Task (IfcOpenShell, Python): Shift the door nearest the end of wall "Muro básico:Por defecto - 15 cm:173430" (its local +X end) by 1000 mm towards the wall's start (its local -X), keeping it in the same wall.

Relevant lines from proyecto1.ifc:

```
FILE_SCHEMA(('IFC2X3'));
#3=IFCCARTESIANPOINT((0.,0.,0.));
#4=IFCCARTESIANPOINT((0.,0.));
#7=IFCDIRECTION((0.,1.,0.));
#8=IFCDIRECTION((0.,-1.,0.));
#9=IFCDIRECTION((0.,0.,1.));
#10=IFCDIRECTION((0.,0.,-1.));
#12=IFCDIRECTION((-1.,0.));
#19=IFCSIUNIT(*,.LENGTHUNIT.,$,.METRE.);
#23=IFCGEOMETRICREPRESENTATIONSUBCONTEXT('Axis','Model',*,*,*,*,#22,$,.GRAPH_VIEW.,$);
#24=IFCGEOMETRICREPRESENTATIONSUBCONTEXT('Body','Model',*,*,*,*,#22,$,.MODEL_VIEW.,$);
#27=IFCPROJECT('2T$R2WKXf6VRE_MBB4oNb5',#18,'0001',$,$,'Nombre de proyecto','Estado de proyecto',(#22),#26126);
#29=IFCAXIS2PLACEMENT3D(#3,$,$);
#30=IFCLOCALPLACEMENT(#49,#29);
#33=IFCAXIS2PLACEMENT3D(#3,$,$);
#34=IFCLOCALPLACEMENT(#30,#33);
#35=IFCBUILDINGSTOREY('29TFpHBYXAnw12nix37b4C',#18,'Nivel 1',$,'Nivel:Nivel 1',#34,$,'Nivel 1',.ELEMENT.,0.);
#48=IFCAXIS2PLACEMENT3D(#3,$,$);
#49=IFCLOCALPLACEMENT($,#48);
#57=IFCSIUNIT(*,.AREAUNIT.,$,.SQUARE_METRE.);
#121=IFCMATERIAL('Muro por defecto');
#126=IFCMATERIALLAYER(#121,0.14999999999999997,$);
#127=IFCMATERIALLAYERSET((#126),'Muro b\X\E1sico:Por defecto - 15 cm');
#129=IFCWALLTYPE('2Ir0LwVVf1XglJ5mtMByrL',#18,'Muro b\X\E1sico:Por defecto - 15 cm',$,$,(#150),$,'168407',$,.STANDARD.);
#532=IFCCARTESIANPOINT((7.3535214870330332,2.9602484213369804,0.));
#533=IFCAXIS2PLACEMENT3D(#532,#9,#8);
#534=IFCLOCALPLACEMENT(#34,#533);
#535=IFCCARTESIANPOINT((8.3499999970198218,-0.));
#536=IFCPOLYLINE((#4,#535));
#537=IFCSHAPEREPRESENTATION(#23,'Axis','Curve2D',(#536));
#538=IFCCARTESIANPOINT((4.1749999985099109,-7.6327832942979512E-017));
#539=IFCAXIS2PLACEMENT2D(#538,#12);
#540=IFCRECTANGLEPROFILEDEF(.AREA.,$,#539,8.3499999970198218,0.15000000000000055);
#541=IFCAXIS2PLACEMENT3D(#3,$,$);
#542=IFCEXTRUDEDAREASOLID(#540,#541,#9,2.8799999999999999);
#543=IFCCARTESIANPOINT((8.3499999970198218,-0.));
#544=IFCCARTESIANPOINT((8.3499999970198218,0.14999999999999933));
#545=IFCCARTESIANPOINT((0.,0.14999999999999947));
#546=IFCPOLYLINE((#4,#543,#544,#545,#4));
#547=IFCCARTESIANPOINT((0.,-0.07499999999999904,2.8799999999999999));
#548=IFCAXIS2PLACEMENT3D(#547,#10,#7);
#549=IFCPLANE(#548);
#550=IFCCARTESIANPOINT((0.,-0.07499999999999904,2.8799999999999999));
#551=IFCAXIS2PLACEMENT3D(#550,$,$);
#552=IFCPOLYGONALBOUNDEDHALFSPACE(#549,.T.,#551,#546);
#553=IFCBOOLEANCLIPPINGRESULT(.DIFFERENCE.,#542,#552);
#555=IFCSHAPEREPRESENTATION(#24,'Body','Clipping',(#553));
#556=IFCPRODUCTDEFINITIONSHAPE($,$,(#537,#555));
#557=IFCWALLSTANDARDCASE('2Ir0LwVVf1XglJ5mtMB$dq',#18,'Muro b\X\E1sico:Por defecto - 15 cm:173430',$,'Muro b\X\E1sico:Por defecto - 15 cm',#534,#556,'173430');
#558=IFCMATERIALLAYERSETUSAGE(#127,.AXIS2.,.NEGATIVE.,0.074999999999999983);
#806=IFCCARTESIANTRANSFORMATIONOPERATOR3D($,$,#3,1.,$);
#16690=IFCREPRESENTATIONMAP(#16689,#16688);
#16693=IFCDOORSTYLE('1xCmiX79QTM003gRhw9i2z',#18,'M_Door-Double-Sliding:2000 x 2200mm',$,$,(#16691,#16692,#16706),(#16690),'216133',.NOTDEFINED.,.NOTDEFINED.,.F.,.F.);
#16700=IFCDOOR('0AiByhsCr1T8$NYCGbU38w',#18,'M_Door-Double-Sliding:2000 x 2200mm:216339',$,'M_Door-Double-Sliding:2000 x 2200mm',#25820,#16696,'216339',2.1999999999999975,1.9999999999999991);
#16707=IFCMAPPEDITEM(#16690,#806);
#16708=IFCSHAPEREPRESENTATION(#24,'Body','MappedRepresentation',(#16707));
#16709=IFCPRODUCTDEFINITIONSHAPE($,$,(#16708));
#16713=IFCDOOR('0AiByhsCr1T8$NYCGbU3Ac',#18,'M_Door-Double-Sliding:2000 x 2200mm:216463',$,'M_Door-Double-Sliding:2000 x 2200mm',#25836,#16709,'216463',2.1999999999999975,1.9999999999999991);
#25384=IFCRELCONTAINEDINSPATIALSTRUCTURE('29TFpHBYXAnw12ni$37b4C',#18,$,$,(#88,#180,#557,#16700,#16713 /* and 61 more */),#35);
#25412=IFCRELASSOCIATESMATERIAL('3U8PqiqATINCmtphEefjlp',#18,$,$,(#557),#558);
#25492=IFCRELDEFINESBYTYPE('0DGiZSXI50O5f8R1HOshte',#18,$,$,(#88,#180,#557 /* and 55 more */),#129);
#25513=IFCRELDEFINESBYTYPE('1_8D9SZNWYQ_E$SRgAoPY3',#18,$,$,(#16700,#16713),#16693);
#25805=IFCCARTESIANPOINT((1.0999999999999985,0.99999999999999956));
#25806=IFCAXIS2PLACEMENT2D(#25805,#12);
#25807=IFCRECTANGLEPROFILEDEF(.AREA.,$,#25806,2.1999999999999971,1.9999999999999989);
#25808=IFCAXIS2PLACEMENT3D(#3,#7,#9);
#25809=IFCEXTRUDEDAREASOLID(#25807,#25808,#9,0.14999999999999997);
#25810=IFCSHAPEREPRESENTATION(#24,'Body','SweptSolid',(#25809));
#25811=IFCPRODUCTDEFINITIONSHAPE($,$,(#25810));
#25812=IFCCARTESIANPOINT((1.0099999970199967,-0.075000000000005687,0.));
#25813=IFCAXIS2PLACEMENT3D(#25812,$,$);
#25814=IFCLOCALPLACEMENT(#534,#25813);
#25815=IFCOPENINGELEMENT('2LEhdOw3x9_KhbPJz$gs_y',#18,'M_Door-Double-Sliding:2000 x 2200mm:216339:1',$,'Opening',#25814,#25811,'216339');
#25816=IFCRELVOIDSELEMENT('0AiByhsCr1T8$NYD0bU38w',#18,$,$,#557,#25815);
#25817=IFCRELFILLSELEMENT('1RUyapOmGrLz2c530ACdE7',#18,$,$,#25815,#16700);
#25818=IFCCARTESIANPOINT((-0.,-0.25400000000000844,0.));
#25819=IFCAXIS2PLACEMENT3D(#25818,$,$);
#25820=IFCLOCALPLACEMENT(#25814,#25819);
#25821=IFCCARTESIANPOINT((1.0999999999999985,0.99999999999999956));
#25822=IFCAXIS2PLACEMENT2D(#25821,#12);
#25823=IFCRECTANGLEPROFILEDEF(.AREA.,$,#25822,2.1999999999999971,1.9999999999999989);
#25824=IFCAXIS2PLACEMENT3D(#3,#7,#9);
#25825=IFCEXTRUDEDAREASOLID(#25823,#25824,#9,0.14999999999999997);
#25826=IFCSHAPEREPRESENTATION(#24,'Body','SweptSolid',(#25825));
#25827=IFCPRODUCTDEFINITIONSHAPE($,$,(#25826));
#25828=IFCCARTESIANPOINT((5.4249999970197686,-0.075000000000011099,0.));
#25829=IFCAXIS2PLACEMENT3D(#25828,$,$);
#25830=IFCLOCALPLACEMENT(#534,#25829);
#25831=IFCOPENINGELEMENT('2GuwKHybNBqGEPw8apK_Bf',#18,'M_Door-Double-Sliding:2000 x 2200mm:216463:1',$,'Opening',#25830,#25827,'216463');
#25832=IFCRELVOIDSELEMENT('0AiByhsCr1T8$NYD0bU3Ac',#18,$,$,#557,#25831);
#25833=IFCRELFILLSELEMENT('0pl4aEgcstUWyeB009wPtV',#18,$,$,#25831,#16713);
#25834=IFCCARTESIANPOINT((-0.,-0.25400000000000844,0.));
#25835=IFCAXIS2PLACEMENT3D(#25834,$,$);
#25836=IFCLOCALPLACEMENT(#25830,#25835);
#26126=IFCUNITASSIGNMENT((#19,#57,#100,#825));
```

```python
import ifcopenshell
import ifcopenshell.api.geometry
import ifcopenshell.util.placement
import ifcopenshell.util.unit

model = ifcopenshell.open("proyecto1.ifc")
unit_scale = ifcopenshell.util.unit.calculate_unit_scale(model)

door = model.by_guid("0AiByhsCr1T8$NYCGbU3Ac")
opening = door.FillsVoids[0].RelatingOpeningElement
wall = opening.VoidsElements[0].RelatingBuildingElement

wall_matrix = ifcopenshell.util.placement.get_local_placement(wall.ObjectPlacement)
shift = wall_matrix[:3, 0] * -1 / unit_scale
before = ifcopenshell.util.placement.get_local_placement(door.ObjectPlacement)[:3, 3].copy()

# The door is placed relative to its opening, so it follows when the opening moves.
matrix = ifcopenshell.util.placement.get_local_placement(opening.ObjectPlacement)
matrix[:3, 3] += shift
ifcopenshell.api.geometry.edit_object_placement(
    model, product=opening, matrix=matrix, is_si=False, should_transform_children=True
)

after = ifcopenshell.util.placement.get_local_placement(door.ObjectPlacement)[:3, 3]
print("door moved by", (after - before).round(3) + 0.0)

model.write("proyecto1_edited.ifc")
```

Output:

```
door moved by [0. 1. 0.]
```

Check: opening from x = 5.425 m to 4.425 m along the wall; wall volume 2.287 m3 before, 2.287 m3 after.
